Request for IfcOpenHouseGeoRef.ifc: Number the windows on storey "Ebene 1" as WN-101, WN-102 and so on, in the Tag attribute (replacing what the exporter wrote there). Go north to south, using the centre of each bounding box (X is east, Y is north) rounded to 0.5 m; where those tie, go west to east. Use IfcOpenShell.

First a look at what the model holds.

```python
import ifcopenshell
import ifcopenshell.util.element
import ifcopenshell.util.placement

model = ifcopenshell.open("IfcOpenHouseGeoRef.ifc")
print(model.schema)
storey = next(s for s in model.by_type("IfcBuildingStorey") if s.Name == "Ebene 1")
windows = [e for e in ifcopenshell.util.element.get_decomposition(storey) if e.is_a("IfcWindow")]
for e in sorted(windows, key=lambda e: e.id()):
    origin = ifcopenshell.util.placement.get_local_placement(e.ObjectPlacement)[:3, 3]
    print(e.id(), e.Tag, e.Name, origin.round(2) + 0.0, sep=" | ")
```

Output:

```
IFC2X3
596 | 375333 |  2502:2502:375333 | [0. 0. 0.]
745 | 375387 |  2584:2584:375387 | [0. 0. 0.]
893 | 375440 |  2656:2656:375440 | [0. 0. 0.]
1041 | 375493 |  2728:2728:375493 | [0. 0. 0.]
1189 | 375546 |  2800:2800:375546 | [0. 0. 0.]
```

```python
import ifcopenshell
import ifcopenshell.geom
import ifcopenshell.util.element
import ifcopenshell.util.shape

model = ifcopenshell.open("IfcOpenHouseGeoRef.ifc")
settings = ifcopenshell.geom.settings()
settings.set("use-world-coords", True)


def centre(element):
    shape = ifcopenshell.geom.create_shape(settings, element)
    return ifcopenshell.util.shape.get_bbox_centroid(shape.geometry)


storey = next(s for s in model.by_type("IfcBuildingStorey") if s.Name == "Ebene 1")
windows = [e for e in ifcopenshell.util.element.get_decomposition(storey) if e.is_a("IfcWindow")]

# Insertion points can sit at a corner or the storey origin, so sort by the geometry (in metres).
centres = {e: centre(e) for e in windows}
windows.sort(key=lambda e: (-round(centres[e][1] / 0.5), centres[e][0]))

for i, e in enumerate(windows, start=1):
    number = f"WN-1{i:02d}"
    e.Tag = number
    print(e.id(), number)

model.write("IfcOpenHouseGeoRef_updated.ifc")
```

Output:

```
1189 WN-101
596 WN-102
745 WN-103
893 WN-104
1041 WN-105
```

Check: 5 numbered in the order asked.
